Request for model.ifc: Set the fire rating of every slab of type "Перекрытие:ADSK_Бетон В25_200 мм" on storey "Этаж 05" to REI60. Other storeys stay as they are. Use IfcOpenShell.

First a look at what the model holds.

```python
import ifcopenshell
import ifcopenshell.util.element

model = ifcopenshell.open("model.ifc")
print(model.schema)
storey = next(s for s in model.by_type("IfcBuildingStorey") if s.Name == "Этаж 05")
slabs = [e for e in ifcopenshell.util.element.get_decomposition(storey) if e.is_a("IfcSlab")]
seen = {}
for e in slabs:
    element_type = ifcopenshell.util.element.get_type(e)
    key = (element_type.Name if element_type != e and element_type else None, ifcopenshell.util.element.get_pset(e, "Pset_SlabCommon", "FireRating"))
    seen[key] = seen.get(key, 0) + 1
for (name, value), count in sorted(seen.items(), key=str):
    print(count, "x", name, "|", value)
```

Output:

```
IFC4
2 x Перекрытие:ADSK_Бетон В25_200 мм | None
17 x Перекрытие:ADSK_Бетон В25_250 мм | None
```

```python
import ifcopenshell
import ifcopenshell.api.pset
import ifcopenshell.util.element

model = ifcopenshell.open("model.ifc")

storey = next(s for s in model.by_type("IfcBuildingStorey") if s.Name == "Этаж 05")
slabs = [e for e in ifcopenshell.util.element.get_decomposition(storey) if e.is_a("IfcSlab")]

count = 0
for e in slabs:
    element_type = ifcopenshell.util.element.get_type(e)
    if element_type in (None, e) or element_type.Name != "Перекрытие:ADSK_Бетон В25_200 мм":
        continue
    # add_pset returns the element's existing set when there is one.
    pset = ifcopenshell.api.pset.add_pset(model, product=e, name="Pset_SlabCommon")
    ifcopenshell.api.pset.edit_pset(model, pset=pset, properties={"FireRating": "REI60"})
    count += 1

print(count, "slabs updated")

model.write("model_updated.ifc")
```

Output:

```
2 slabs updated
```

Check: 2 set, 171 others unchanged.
